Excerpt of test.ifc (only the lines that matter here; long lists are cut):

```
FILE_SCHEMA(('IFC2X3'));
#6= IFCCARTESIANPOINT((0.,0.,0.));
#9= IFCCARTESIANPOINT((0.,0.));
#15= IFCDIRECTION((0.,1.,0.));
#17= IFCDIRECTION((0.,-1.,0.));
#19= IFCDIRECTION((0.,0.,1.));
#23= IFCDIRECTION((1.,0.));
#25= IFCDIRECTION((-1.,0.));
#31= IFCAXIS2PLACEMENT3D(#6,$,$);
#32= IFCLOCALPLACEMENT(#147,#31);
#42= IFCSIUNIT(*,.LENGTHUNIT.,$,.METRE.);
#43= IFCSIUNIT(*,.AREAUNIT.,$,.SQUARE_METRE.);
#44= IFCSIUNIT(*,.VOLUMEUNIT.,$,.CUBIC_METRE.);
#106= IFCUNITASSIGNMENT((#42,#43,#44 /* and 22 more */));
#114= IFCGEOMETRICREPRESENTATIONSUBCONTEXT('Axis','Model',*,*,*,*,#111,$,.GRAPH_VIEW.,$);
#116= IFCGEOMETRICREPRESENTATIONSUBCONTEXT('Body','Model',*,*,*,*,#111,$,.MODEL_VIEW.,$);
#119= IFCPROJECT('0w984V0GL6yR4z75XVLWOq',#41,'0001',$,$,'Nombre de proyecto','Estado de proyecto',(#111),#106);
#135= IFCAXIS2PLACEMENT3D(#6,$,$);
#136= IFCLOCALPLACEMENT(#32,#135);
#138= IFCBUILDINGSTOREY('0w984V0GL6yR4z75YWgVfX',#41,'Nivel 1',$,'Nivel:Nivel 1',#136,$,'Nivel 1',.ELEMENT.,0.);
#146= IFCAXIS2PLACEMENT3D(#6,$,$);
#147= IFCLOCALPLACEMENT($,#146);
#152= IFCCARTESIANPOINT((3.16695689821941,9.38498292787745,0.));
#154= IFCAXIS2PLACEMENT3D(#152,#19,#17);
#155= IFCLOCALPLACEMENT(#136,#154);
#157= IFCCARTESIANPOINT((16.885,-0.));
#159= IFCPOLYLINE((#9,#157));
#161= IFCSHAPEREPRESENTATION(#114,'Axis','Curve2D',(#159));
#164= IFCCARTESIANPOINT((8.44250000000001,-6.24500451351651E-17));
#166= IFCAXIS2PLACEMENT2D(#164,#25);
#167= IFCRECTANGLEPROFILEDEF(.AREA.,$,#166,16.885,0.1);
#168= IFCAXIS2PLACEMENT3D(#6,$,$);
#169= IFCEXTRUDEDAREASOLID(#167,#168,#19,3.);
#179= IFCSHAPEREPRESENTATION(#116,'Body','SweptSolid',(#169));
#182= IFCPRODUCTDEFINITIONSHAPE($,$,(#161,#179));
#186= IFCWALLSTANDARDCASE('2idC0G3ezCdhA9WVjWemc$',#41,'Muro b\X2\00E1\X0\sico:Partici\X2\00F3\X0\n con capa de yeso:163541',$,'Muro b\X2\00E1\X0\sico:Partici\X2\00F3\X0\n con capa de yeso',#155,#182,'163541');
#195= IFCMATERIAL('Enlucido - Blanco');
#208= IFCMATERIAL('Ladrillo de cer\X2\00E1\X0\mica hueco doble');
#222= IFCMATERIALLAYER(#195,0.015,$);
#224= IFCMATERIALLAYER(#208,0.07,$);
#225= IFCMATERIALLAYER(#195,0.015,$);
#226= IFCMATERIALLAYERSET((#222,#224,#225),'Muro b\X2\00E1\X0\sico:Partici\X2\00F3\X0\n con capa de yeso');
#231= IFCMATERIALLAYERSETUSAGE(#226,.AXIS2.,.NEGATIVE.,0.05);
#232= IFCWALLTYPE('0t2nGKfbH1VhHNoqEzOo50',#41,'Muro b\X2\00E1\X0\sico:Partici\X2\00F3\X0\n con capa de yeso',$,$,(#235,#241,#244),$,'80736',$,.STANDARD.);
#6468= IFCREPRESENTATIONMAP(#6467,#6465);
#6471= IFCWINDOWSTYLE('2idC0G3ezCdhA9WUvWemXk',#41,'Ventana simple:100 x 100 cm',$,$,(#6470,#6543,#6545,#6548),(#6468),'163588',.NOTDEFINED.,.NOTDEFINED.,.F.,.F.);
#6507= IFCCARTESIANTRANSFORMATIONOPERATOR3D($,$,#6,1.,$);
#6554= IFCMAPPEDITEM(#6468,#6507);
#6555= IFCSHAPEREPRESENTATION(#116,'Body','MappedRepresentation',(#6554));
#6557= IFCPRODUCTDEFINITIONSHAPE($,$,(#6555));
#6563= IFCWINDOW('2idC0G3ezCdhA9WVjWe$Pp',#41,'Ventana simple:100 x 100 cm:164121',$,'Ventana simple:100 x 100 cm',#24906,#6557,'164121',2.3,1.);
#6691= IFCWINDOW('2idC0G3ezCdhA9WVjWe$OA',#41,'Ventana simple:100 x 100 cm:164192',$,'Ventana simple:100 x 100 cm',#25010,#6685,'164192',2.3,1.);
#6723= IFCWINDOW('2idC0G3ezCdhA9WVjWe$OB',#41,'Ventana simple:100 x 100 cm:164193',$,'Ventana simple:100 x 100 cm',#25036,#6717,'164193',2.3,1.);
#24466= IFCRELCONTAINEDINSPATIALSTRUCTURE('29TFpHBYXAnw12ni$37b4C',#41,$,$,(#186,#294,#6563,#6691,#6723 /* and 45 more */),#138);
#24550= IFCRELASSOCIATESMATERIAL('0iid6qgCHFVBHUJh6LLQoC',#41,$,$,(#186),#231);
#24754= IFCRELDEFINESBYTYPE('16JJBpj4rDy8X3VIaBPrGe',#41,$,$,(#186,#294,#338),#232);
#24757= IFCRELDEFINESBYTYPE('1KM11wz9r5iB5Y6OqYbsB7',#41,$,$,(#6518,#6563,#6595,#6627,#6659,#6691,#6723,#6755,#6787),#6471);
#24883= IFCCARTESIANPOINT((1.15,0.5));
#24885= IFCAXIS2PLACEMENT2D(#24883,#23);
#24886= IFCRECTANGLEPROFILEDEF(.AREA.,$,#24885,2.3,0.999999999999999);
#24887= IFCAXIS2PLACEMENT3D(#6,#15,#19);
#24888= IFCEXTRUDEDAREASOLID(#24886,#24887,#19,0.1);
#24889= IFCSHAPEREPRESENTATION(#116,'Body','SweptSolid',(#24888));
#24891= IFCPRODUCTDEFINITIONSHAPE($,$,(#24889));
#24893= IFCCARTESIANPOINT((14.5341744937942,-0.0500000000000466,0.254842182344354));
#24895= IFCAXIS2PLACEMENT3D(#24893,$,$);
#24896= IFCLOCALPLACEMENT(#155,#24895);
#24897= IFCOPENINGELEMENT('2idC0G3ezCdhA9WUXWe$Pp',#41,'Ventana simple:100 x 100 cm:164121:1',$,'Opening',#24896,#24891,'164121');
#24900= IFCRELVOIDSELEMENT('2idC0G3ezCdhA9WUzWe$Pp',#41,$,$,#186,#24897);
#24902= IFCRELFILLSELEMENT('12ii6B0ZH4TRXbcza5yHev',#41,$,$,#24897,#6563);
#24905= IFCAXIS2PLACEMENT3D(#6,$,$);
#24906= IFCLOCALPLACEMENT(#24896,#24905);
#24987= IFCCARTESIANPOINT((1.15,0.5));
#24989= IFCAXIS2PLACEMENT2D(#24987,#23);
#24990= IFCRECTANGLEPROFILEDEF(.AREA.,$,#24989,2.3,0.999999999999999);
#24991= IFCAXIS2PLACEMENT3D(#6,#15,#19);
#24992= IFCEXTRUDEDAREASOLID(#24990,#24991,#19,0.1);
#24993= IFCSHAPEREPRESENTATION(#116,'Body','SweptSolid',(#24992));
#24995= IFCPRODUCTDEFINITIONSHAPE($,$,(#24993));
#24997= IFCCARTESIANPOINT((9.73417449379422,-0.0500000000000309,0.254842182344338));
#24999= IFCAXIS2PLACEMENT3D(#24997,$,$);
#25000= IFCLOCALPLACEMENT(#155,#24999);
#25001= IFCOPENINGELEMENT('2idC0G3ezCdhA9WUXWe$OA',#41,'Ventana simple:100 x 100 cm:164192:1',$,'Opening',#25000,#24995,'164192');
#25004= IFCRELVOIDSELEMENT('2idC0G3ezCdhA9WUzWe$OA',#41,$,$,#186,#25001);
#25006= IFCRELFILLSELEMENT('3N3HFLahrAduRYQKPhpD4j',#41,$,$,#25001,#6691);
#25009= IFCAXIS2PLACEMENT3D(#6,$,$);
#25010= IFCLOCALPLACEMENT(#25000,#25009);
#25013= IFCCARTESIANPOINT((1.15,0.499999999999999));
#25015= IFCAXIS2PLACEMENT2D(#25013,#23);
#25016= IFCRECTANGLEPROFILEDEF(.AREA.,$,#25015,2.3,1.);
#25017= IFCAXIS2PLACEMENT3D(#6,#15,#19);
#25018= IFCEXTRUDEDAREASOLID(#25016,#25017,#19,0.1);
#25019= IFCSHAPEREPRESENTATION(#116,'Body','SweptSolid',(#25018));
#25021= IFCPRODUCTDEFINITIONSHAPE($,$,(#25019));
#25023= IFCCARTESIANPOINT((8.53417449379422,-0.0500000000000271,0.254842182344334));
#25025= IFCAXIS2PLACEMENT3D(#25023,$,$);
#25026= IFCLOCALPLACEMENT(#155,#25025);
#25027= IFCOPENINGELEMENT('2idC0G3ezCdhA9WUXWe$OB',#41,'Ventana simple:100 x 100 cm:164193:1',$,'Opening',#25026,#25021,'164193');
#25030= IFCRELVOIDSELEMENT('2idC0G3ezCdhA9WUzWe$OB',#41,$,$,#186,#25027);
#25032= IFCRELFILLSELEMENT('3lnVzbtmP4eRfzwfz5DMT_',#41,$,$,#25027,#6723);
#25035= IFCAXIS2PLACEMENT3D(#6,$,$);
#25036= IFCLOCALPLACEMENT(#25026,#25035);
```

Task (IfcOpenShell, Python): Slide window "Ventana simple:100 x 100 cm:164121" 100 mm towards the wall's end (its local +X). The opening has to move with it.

```python
import ifcopenshell
import ifcopenshell.api.geometry
import ifcopenshell.util.placement
import ifcopenshell.util.unit

model = ifcopenshell.open("test.ifc")
unit_scale = ifcopenshell.util.unit.calculate_unit_scale(model)

window = model.by_guid("2idC0G3ezCdhA9WVjWe$Pp")
opening = window.FillsVoids[0].RelatingOpeningElement
wall = opening.VoidsElements[0].RelatingBuildingElement

wall_matrix = ifcopenshell.util.placement.get_local_placement(wall.ObjectPlacement)
shift = wall_matrix[:3, 0] * 0.1 / unit_scale
before = ifcopenshell.util.placement.get_local_placement(window.ObjectPlacement)[:3, 3].copy()

# The window is placed relative to its opening, so it follows when the opening moves.
matrix = ifcopenshell.util.placement.get_local_placement(opening.ObjectPlacement)
matrix[:3, 3] += shift
ifcopenshell.api.geometry.edit_object_placement(
    model, product=opening, matrix=matrix, is_si=False, should_transform_children=True
)

after = ifcopenshell.util.placement.get_local_placement(window.ObjectPlacement)[:3, 3]
print("window moved by", (after - before).round(3) + 0.0)

model.write("test_edited.ifc")
```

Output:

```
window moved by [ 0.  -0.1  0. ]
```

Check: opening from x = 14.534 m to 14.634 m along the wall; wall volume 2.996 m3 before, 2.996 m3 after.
